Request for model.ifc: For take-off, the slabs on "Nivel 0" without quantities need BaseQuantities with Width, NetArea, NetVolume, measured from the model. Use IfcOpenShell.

First a look at what the model holds.

```python
import ifcopenshell
import ifcopenshell.util.element
import ifcopenshell.util.unit

model = ifcopenshell.open("model.ifc")
print(model.schema)
for unit_type in ("LENGTHUNIT", "AREAUNIT", "VOLUMEUNIT"):
    print(unit_type, ifcopenshell.util.unit.calculate_unit_scale(model, unit_type))
storey = next(s for s in model.by_type("IfcBuildingStorey") if s.Name == "Nivel 0")
slabs = [e for e in ifcopenshell.util.element.get_decomposition(storey) if e.is_a("IfcSlab")]
for e in sorted(slabs, key=lambda e: e.id()):
    print(e.id(), e.is_a(), e.Name, list(ifcopenshell.util.element.get_psets(e, qtos_only=True)), sep=" | ")
```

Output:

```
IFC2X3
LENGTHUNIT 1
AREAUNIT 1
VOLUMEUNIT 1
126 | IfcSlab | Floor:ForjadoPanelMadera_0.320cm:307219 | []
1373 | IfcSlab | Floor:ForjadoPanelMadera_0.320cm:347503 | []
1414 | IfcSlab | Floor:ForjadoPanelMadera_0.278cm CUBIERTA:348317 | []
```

```python
import ifcopenshell
import ifcopenshell.api.pset
import ifcopenshell.geom
import ifcopenshell.util.element
import ifcopenshell.util.shape
import ifcopenshell.util.unit

model = ifcopenshell.open("model.ifc")
unit_scale = ifcopenshell.util.unit.calculate_unit_scale(model)
area_scale = ifcopenshell.util.unit.calculate_unit_scale(model, "AREAUNIT")
volume_scale = ifcopenshell.util.unit.calculate_unit_scale(model, "VOLUMEUNIT")
settings = ifcopenshell.geom.settings()

storey = next(s for s in model.by_type("IfcBuildingStorey") if s.Name == "Nivel 0")
slabs = [e for e in ifcopenshell.util.element.get_decomposition(storey) if e.is_a("IfcSlab")]

for e in sorted(slabs, key=lambda e: e.id()):
    if ifcopenshell.util.element.get_psets(e, qtos_only=True, should_inherit=False):
        continue
    # Geometry comes back in metres, in the element's own axes.
    shape = ifcopenshell.geom.create_shape(settings, e)
    values = {
        "Width": ifcopenshell.util.shape.get_z(shape.geometry) / unit_scale,
        "NetArea": ifcopenshell.util.shape.get_footprint_area(shape.geometry) / area_scale,
        "NetVolume": ifcopenshell.util.shape.get_volume(shape.geometry) / volume_scale,
    }
    qto = ifcopenshell.api.pset.add_qto(model, product=e, name="BaseQuantities")
    ifcopenshell.api.pset.edit_qto(model, qto=qto, properties=values)
    print(e.id(), {k: round(v, 3) for k, v in values.items()})

model.write("model_rev.ifc")
```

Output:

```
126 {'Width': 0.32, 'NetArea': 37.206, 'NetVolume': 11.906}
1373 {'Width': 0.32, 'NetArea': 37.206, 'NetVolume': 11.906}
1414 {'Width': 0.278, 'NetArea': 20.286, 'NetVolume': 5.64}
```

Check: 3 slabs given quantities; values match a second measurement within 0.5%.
